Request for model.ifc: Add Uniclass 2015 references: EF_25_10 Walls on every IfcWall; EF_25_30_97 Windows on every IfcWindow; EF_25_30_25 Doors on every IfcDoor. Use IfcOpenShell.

First a look at what the model holds.

```python
import ifcopenshell

model = ifcopenshell.open("model.ifc")
print(model.schema)
print("classifications:", [c.Name for c in model.by_type("IfcClassification")])
for ifc_class in ("IfcDoor", "IfcRoof", "IfcStair", "IfcWall", "IfcWindow"):
    print(ifc_class, len(model.by_type(ifc_class)))
```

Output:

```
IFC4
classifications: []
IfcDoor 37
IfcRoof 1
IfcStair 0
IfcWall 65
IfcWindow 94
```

```python
import ifcopenshell
import ifcopenshell.api.classification

model = ifcopenshell.open("model.ifc")

system = ifcopenshell.api.classification.add_classification(model, classification="Uniclass 2015")

codes = {
    "IfcWall": ("EF_25_10", "Walls"),
    "IfcWindow": ("EF_25_30_97", "Windows"),
    "IfcDoor": ("EF_25_30_25", "Doors"),
}
for ifc_class, (code, name) in codes.items():
    products = model.by_type(ifc_class)
    ifcopenshell.api.classification.add_reference(
        model, products=products, classification=system, identification=code, name=name
    )
    print(code, len(products))

model.write("model_v2.ifc")
```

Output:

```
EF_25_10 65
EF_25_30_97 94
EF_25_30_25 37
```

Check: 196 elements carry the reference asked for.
